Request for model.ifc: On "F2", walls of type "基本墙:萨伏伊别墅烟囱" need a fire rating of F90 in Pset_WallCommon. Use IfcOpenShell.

First a look at what the model holds.

```python
import ifcopenshell
import ifcopenshell.util.element

model = ifcopenshell.open("model.ifc")
print(model.schema)
storey = next(s for s in model.by_type("IfcBuildingStorey") if s.Name == "F2")
walls = [e for e in ifcopenshell.util.element.get_decomposition(storey) if e.is_a("IfcWall")]
seen = {}
for e in walls:
    element_type = ifcopenshell.util.element.get_type(e)
    key = (element_type.Name if element_type != e and element_type else None, ifcopenshell.util.element.get_pset(e, "Pset_WallCommon", "FireRating"))
    seen[key] = seen.get(key, 0) + 1
for (name, value), count in sorted(seen.items(), key=str):
    print(count, "x", name, "|", value)
```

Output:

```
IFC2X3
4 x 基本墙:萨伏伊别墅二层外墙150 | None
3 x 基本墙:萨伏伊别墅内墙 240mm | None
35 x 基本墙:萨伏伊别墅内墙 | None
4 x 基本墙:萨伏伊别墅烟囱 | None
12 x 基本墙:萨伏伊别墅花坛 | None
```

```python
import ifcopenshell
import ifcopenshell.api.pset
import ifcopenshell.util.element

model = ifcopenshell.open("model.ifc")

storey = next(s for s in model.by_type("IfcBuildingStorey") if s.Name == "F2")
walls = [e for e in ifcopenshell.util.element.get_decomposition(storey) if e.is_a("IfcWall")]

count = 0
for e in walls:
    element_type = ifcopenshell.util.element.get_type(e)
    if element_type in (None, e) or element_type.Name != "基本墙:萨伏伊别墅烟囱":
        continue
    # add_pset returns the element's existing set when there is one.
    pset = ifcopenshell.api.pset.add_pset(model, product=e, name="Pset_WallCommon")
    ifcopenshell.api.pset.edit_pset(model, pset=pset, properties={"FireRating": "F90"})
    count += 1

print(count, "walls updated")

model.write("model_updated.ifc")
```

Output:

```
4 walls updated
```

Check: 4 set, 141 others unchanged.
